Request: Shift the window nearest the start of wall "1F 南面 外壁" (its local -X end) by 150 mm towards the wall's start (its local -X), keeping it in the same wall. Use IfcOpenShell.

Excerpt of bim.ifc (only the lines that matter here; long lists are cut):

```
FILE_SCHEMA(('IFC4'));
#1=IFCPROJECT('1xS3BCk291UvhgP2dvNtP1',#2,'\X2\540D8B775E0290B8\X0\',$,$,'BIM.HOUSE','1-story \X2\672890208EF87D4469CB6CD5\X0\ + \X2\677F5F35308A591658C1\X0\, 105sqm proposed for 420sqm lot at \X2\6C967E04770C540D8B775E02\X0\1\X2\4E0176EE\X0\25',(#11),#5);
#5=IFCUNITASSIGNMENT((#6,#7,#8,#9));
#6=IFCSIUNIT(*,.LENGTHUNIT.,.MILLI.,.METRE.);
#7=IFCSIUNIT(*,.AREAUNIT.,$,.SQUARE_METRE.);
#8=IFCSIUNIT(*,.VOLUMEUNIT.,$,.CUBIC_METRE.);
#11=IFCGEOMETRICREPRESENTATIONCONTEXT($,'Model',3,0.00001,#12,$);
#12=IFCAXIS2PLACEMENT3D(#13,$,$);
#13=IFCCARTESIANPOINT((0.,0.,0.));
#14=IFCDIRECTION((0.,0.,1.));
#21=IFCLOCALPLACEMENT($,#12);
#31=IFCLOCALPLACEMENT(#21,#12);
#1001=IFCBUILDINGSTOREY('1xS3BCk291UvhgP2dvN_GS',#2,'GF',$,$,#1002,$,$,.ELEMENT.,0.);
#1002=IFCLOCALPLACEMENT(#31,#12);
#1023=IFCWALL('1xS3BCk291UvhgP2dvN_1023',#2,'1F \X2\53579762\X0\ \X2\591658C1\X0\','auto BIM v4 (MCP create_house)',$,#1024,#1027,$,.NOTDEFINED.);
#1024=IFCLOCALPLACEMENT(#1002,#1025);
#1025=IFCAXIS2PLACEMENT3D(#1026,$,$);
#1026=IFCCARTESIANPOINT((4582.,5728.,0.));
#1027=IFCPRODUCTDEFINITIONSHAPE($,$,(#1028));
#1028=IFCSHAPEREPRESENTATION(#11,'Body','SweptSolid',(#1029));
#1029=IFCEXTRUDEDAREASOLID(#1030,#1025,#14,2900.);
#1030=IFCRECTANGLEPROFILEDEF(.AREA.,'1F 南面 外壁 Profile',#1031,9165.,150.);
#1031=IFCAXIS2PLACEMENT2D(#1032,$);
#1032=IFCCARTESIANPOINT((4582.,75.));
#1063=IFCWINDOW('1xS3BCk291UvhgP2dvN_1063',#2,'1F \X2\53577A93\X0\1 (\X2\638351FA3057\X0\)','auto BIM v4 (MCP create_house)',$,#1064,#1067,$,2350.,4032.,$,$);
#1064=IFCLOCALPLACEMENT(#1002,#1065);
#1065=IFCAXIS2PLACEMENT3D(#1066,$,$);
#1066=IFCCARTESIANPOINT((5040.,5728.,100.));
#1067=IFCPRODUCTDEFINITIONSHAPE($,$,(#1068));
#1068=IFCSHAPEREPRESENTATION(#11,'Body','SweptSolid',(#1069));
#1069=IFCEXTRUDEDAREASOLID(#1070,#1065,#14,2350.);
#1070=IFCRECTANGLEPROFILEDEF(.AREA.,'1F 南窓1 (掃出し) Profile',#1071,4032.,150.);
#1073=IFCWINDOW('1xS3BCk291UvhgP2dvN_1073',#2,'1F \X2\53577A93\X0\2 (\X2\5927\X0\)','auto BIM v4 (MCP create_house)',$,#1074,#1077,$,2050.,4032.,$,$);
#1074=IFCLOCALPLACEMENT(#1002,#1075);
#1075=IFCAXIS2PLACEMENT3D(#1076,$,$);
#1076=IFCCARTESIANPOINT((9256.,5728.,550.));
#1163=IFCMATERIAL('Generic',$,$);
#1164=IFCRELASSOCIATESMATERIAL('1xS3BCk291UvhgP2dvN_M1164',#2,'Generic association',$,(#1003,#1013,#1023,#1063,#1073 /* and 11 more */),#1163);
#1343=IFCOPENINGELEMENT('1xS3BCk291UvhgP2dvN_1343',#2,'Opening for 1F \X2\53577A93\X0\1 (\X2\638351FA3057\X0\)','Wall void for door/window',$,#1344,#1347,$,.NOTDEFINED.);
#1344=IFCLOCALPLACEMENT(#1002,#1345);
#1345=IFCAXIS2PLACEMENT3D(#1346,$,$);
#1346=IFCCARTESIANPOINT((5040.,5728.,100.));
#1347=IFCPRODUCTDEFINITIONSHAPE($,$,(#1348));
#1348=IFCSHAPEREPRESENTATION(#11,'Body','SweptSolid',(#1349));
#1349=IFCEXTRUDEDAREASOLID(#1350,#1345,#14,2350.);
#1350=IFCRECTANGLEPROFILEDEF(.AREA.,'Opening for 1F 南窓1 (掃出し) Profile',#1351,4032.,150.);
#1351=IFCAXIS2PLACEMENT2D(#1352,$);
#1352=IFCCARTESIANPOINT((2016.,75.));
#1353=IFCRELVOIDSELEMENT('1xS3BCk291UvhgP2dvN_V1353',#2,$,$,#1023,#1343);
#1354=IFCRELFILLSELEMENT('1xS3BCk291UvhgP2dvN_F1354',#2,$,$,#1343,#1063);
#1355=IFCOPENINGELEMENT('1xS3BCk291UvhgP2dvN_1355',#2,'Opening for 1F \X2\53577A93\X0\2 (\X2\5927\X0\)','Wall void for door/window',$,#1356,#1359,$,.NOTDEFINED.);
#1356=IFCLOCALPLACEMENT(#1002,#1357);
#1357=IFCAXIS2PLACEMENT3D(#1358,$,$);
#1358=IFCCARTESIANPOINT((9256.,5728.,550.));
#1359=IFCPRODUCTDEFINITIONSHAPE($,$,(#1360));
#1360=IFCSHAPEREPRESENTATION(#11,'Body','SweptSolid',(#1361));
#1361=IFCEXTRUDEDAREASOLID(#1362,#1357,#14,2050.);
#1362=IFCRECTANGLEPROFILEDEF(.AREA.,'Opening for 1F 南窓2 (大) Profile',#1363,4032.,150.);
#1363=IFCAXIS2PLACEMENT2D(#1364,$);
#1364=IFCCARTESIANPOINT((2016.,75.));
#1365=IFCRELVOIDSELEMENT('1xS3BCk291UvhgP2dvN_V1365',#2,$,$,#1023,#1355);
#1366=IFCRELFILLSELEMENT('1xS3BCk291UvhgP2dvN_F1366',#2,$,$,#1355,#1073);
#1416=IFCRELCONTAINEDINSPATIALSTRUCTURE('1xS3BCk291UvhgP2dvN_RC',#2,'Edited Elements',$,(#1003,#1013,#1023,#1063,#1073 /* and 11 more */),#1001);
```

```python
import ifcopenshell
import ifcopenshell.api.geometry
import ifcopenshell.util.placement
import ifcopenshell.util.unit

model = ifcopenshell.open("bim.ifc")
unit_scale = ifcopenshell.util.unit.calculate_unit_scale(model)

window = model.by_id(1063)
opening = window.FillsVoids[0].RelatingOpeningElement
wall = opening.VoidsElements[0].RelatingBuildingElement

wall_matrix = ifcopenshell.util.placement.get_local_placement(wall.ObjectPlacement)
shift = wall_matrix[:3, 0] * -0.15 / unit_scale
before = ifcopenshell.util.placement.get_local_placement(window.ObjectPlacement)[:3, 3].copy()

# The window is not placed relative to its opening, so move both.
for product in (opening, window):
    matrix = ifcopenshell.util.placement.get_local_placement(product.ObjectPlacement)
    matrix[:3, 3] += shift
    ifcopenshell.api.geometry.edit_object_placement(model, product=product, matrix=matrix, is_si=False)

after = ifcopenshell.util.placement.get_local_placement(window.ObjectPlacement)[:3, 3]
print("window moved by", (after - before).round(3) + 0.0)

model.write("bim_rev.ifc")
```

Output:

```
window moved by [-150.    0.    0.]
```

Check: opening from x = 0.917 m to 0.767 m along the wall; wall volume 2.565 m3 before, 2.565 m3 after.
